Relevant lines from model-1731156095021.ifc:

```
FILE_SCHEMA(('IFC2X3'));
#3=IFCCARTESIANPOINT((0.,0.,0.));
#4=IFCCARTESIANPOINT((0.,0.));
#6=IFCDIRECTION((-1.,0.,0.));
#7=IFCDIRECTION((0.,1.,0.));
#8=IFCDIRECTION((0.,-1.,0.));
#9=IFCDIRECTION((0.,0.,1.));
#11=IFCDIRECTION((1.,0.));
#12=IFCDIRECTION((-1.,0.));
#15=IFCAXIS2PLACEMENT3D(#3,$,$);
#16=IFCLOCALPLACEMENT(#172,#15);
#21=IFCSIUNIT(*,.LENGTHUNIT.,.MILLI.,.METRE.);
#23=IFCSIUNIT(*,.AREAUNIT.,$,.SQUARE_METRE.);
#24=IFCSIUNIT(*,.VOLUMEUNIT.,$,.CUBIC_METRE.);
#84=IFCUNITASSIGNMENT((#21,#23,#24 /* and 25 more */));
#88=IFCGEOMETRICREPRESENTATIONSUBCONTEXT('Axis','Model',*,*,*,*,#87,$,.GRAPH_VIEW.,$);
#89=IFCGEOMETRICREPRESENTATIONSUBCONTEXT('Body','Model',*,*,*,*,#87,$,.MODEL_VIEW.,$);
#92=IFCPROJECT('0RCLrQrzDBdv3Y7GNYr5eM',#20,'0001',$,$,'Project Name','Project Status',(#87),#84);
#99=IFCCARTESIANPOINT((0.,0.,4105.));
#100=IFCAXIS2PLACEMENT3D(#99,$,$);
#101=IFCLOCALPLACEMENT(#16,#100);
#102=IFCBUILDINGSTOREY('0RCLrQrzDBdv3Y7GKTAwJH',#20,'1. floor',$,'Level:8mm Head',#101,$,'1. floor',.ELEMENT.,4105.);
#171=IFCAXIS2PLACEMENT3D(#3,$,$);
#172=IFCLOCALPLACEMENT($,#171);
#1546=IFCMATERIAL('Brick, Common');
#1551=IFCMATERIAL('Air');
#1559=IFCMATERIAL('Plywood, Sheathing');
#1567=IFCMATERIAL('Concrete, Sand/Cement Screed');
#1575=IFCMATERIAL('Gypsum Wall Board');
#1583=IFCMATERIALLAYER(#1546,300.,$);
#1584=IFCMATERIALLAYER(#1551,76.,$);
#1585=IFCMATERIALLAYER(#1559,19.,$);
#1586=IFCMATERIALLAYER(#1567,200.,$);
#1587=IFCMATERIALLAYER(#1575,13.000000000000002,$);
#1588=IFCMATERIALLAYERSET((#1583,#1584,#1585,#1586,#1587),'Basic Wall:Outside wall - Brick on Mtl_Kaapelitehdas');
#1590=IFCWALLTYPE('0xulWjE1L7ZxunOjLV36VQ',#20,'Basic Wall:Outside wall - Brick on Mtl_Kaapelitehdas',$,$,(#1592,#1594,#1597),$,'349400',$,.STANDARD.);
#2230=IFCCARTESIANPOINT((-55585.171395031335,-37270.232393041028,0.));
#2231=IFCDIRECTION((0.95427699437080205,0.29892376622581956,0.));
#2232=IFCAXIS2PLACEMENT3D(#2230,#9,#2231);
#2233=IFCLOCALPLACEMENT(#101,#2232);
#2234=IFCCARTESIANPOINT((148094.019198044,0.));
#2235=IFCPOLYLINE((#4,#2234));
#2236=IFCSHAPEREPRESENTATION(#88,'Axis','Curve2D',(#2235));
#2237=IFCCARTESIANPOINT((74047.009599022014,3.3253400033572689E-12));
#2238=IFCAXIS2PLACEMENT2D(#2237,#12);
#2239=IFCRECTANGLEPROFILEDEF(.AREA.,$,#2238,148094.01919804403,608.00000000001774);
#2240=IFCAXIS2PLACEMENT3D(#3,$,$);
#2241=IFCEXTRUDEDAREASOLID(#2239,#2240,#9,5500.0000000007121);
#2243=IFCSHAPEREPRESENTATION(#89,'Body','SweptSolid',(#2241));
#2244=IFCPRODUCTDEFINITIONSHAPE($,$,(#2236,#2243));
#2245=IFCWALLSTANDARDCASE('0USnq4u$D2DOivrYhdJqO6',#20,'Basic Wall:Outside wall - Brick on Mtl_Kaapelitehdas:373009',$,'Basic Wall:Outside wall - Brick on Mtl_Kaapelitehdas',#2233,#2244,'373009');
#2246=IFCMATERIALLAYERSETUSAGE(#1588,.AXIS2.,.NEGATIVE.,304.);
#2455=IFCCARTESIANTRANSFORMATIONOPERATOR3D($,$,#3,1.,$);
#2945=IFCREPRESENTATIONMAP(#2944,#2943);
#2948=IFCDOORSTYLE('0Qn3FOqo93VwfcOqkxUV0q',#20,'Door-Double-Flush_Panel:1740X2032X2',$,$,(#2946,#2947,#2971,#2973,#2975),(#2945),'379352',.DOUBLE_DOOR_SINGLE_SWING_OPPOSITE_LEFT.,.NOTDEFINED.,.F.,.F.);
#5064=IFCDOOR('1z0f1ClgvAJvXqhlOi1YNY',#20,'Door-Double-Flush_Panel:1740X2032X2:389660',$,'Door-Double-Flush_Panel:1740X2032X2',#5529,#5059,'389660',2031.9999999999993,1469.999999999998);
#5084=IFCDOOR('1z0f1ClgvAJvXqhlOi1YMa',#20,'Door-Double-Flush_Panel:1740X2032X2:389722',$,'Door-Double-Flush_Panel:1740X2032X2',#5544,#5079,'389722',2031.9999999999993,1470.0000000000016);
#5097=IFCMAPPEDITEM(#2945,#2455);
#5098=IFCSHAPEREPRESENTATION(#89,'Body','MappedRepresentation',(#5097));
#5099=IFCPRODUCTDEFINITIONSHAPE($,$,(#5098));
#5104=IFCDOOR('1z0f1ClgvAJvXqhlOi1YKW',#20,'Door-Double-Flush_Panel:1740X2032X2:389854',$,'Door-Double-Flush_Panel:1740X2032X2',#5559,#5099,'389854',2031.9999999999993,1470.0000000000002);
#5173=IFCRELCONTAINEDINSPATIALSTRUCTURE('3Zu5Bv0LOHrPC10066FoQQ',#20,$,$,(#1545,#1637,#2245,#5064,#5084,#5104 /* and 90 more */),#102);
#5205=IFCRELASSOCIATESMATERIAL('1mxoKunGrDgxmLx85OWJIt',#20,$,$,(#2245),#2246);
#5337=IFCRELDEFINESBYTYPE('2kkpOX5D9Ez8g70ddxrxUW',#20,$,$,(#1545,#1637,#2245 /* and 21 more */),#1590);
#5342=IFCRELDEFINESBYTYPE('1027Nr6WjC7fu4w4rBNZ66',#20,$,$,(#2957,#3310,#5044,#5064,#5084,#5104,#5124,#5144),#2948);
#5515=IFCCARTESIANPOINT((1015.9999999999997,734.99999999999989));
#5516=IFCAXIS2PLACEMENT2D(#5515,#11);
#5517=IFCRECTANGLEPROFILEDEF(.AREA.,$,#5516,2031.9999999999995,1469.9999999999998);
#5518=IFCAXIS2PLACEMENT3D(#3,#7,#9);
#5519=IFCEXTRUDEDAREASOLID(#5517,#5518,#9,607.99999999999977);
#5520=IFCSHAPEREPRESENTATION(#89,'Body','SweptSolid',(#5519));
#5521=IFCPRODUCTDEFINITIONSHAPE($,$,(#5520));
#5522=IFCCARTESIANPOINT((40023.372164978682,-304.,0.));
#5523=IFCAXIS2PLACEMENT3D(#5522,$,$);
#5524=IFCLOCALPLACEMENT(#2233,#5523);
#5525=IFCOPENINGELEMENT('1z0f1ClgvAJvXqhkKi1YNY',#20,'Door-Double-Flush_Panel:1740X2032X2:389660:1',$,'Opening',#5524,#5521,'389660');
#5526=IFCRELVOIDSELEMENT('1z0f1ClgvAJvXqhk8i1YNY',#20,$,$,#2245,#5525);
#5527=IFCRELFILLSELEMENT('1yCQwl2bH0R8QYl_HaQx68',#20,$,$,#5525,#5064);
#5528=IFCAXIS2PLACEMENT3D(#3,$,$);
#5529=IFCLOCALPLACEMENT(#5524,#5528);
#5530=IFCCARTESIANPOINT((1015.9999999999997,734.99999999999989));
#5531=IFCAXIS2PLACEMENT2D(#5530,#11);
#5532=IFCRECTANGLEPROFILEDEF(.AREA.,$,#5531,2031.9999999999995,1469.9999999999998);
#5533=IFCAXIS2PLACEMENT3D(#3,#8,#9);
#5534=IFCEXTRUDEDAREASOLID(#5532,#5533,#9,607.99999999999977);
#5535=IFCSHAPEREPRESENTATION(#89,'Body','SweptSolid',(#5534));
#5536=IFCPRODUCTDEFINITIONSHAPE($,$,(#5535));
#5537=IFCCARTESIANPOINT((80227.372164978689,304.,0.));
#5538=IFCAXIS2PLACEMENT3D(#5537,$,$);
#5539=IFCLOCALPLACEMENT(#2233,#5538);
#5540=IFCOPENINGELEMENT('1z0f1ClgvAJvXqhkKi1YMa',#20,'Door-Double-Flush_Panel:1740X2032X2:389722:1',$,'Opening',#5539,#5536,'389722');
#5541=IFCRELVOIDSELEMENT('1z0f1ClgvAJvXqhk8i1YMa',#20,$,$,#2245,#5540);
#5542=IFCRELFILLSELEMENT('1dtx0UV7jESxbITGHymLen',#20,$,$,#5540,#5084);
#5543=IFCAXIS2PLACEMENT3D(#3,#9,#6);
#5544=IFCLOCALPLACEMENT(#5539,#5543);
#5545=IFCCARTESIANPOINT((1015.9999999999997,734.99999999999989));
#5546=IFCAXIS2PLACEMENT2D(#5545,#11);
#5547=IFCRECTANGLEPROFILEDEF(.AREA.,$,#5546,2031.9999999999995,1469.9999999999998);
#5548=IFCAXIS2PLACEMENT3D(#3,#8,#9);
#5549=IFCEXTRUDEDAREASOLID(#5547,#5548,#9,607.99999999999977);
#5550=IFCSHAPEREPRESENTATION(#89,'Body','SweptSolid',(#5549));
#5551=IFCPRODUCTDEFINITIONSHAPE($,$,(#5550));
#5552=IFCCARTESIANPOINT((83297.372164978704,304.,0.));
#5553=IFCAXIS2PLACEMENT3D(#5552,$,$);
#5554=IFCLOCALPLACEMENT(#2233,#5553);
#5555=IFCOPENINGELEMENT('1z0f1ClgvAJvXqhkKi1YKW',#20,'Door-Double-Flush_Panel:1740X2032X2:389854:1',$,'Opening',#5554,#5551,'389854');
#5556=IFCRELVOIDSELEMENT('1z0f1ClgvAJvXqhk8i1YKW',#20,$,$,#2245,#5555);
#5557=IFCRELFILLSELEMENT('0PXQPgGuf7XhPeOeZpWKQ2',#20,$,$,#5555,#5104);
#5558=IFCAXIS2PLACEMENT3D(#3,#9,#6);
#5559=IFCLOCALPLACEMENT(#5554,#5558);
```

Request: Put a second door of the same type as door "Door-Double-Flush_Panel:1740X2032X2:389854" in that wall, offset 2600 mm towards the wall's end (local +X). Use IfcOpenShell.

```python
import ifcopenshell
import ifcopenshell.api.feature
import ifcopenshell.api.geometry
import ifcopenshell.api.root
import ifcopenshell.geom
import ifcopenshell.util.element
import ifcopenshell.util.placement
import ifcopenshell.util.shape

model = ifcopenshell.open("model-1731156095021.ifc")
settings = ifcopenshell.geom.settings()


def volume(element):
    """Net volume in cubic metres, openings subtracted."""
    shape = ifcopenshell.geom.create_shape(settings, element)
    return ifcopenshell.util.shape.get_volume(shape.geometry)


def reuse_history(source, copy):
    """copy_class also copies each property set's owner history, people and application; keep the originals."""
    for rel in copy.IsDefinedBy:
        if rel.is_a("IfcRelDefinesByProperties") and (history := rel.RelatingPropertyDefinition.OwnerHistory):
            rel.RelatingPropertyDefinition.OwnerHistory = source.OwnerHistory
            ifcopenshell.util.element.remove_deep2(model, history)


door = model.by_guid("1z0f1ClgvAJvXqhlOi1YKW")
opening = door.FillsVoids[0].RelatingOpeningElement
wall = opening.VoidsElements[0].RelatingBuildingElement
before = volume(wall)
shift = ifcopenshell.util.placement.get_local_placement(wall.ObjectPlacement)[:3, 0] * 2600.0

# copy_class copies the void relationship, type, container and properties, but no geometry.
new_opening = ifcopenshell.api.root.copy_class(model, product=opening)
new_opening.Representation = ifcopenshell.util.element.copy_deep(
    model, opening.Representation, exclude=["IfcGeometricRepresentationContext", "IfcRepresentationMap"]
)
new_opening.Name = "Door-Double-Flush_Panel:1740X2032X2"
new_opening.Tag = None
new_door = ifcopenshell.api.root.copy_class(model, product=door)
new_door.Representation = ifcopenshell.util.element.copy_deep(
    model, door.Representation, exclude=["IfcGeometricRepresentationContext", "IfcRepresentationMap"]
)
new_door.Name = "Door-Double-Flush_Panel:1740X2032X2"
new_door.Tag = None
reuse_history(door, new_door)
fills = ifcopenshell.api.feature.add_filling(model, opening=new_opening, element=new_door)
fills.OwnerHistory = new_door.OwnerHistory  # required in IFC2X3

for old, new in ((opening, new_opening), (door, new_door)):
    matrix = ifcopenshell.util.placement.get_local_placement(old.ObjectPlacement)
    matrix[:3, 3] += shift
    ifcopenshell.api.geometry.edit_object_placement(model, product=new, matrix=matrix, is_si=False)

after = volume(wall)

print(f"wall volume {before:.3f} -> {after:.3f} m3")

model.write("model-1731156095021_updated.ifc")
```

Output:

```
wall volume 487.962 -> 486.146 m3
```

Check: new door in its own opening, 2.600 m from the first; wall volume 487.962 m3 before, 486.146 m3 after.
